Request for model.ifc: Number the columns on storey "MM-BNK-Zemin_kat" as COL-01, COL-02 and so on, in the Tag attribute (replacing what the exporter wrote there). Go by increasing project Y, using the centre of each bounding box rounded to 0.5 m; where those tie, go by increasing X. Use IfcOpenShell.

First a look at what the model holds.

```python
import ifcopenshell
import ifcopenshell.util.element
import ifcopenshell.util.placement

model = ifcopenshell.open("model.ifc")
print(model.schema)
storey = next(s for s in model.by_type("IfcBuildingStorey") if s.Name == "MM-BNK-Zemin_kat")
columns = [e for e in ifcopenshell.util.element.get_decomposition(storey) if e.is_a("IfcColumn")]
for e in sorted(columns, key=lambda e: e.id()):
    origin = ifcopenshell.util.placement.get_local_placement(e.ObjectPlacement)[:3, 3]
    print(e.id(), e.Tag, e.Name, origin.round(2) + 0.0, sep=" | ")
```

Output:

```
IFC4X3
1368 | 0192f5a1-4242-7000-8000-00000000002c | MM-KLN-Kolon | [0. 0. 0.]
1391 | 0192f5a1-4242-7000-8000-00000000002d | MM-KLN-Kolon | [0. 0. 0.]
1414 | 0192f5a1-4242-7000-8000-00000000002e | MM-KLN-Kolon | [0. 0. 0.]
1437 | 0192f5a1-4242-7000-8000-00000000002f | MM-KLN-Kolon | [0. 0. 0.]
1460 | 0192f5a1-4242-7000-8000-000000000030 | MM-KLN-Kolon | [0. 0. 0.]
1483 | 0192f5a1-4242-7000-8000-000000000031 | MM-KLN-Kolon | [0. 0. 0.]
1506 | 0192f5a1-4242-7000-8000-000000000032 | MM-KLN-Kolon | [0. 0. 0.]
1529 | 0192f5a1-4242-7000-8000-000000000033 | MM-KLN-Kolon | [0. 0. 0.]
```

```python
import ifcopenshell
import ifcopenshell.geom
import ifcopenshell.util.element
import ifcopenshell.util.shape

model = ifcopenshell.open("model.ifc")
settings = ifcopenshell.geom.settings()
settings.set("use-world-coords", True)


def centre(element):
    shape = ifcopenshell.geom.create_shape(settings, element)
    return ifcopenshell.util.shape.get_bbox_centroid(shape.geometry)


storey = next(s for s in model.by_type("IfcBuildingStorey") if s.Name == "MM-BNK-Zemin_kat")
columns = [e for e in ifcopenshell.util.element.get_decomposition(storey) if e.is_a("IfcColumn")]

# Insertion points can sit at a corner or the storey origin, so sort by the geometry (in metres).
centres = {e: centre(e) for e in columns}
columns.sort(key=lambda e: (round(centres[e][1] / 0.5), centres[e][0]))

for i, e in enumerate(columns, start=1):
    number = f"COL-{i:02d}"
    e.Tag = number
    print(e.id(), number)

model.write("model_edited.ifc")
```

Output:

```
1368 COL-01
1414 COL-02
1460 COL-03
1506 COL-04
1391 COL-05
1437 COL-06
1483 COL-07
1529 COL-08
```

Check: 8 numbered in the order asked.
